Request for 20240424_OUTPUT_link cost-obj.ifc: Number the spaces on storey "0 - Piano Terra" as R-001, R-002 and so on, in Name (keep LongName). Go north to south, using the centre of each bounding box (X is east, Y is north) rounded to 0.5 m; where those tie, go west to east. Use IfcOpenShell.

First a look at what the model holds.

```python
import ifcopenshell
import ifcopenshell.util.element
import ifcopenshell.util.placement

model = ifcopenshell.open("20240424_OUTPUT_link cost-obj.ifc")
print(model.schema)
storey = next(s for s in model.by_type("IfcBuildingStorey") if s.Name == "0 - Piano Terra")
spaces = [e for e in ifcopenshell.util.element.get_decomposition(storey) if e.is_a("IfcSpace")]
for e in sorted(spaces, key=lambda e: e.id()):
    origin = ifcopenshell.util.placement.get_local_placement(e.ObjectPlacement)[:3, 3]
    print(e.id(), e.Name, e.LongName, origin.round(2) + 0.0, sep=" | ")
```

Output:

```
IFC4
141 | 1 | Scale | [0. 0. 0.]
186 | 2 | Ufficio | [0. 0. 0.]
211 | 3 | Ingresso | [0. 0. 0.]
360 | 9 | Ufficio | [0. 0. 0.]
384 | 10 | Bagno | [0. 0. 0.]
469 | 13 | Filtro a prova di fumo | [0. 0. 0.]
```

```python
import ifcopenshell
import ifcopenshell.geom
import ifcopenshell.util.element
import ifcopenshell.util.shape

model = ifcopenshell.open("20240424_OUTPUT_link cost-obj.ifc")
settings = ifcopenshell.geom.settings()
settings.set("use-world-coords", True)


def centre(element):
    shape = ifcopenshell.geom.create_shape(settings, element)
    return ifcopenshell.util.shape.get_bbox_centroid(shape.geometry)


storey = next(s for s in model.by_type("IfcBuildingStorey") if s.Name == "0 - Piano Terra")
spaces = [e for e in ifcopenshell.util.element.get_decomposition(storey) if e.is_a("IfcSpace")]

# Insertion points can sit at a corner or the storey origin, so sort by the geometry (in metres).
centres = {e: centre(e) for e in spaces}
spaces.sort(key=lambda e: (-round(centres[e][1] / 0.5), centres[e][0]))

for i, e in enumerate(spaces, start=1):
    number = f"R-0{i:02d}"
    e.Name = number
    print(e.id(), number)

model.write("20240424_OUTPUT_link cost-obj-out.ifc")
```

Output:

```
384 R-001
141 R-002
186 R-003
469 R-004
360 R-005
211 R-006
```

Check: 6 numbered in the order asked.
